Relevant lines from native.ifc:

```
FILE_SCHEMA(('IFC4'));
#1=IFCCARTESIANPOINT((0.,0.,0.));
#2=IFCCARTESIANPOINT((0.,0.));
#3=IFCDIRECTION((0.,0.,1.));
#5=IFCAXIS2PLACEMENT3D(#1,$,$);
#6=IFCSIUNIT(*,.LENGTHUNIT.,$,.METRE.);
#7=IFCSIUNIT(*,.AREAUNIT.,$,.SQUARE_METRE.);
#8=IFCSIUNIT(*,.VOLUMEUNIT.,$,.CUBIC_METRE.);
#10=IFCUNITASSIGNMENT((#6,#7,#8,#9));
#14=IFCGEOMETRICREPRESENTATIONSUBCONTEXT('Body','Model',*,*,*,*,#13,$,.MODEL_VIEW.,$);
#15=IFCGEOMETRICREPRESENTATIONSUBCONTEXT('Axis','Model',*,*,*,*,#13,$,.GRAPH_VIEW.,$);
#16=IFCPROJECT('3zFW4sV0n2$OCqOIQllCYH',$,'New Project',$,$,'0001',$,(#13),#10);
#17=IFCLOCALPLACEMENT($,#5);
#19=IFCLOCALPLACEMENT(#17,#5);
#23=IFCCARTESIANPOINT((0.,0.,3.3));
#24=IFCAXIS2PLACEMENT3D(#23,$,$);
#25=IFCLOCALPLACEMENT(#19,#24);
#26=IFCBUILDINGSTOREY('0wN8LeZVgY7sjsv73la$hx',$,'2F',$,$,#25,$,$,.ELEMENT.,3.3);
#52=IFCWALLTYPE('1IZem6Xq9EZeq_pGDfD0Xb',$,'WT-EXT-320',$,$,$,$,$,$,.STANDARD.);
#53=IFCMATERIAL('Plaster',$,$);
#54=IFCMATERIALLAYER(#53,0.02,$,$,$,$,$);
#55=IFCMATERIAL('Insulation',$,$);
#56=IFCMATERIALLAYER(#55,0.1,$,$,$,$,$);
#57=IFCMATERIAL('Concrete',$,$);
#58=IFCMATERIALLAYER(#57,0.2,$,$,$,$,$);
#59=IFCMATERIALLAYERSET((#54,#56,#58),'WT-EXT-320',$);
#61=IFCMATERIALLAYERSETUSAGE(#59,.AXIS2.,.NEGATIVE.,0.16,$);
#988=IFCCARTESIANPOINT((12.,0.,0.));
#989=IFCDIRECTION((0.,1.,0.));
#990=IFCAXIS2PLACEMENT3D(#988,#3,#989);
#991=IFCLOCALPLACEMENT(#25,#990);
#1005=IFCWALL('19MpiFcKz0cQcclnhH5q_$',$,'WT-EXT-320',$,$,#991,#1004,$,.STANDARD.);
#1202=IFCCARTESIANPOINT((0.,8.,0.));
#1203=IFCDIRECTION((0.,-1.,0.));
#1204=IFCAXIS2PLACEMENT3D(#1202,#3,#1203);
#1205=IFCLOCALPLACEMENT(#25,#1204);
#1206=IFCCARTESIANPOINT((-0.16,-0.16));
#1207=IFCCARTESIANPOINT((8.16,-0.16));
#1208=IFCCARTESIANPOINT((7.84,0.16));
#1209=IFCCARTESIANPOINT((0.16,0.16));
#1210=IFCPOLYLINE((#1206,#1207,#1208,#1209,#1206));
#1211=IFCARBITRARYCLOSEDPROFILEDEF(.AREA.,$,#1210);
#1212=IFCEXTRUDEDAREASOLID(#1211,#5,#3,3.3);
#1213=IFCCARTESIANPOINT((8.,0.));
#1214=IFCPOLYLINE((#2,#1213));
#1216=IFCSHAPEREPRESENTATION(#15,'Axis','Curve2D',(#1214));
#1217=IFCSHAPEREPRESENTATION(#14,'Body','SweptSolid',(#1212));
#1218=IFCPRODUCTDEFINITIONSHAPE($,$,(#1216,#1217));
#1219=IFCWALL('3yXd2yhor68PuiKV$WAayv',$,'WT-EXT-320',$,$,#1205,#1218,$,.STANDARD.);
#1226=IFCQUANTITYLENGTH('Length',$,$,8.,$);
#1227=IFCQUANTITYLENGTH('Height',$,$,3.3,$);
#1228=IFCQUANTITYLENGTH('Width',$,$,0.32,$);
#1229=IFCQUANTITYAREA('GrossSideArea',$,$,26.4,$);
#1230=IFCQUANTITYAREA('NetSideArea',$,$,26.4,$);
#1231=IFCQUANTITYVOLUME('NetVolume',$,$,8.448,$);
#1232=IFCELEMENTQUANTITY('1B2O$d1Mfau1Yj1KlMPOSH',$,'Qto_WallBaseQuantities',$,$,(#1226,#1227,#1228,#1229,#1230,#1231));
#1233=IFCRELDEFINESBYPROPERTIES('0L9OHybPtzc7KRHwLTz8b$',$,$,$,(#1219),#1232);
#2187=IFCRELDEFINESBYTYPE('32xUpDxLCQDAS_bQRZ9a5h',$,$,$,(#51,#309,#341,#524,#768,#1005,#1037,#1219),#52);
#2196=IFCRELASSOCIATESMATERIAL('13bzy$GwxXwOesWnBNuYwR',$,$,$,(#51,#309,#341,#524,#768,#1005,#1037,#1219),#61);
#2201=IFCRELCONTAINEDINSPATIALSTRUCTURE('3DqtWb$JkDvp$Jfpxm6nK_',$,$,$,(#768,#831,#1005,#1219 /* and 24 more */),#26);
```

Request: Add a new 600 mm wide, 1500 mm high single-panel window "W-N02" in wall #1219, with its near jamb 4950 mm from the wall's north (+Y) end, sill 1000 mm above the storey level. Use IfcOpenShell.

```python
import numpy as np
import ifcopenshell
import ifcopenshell.api.feature
import ifcopenshell.api.geometry
import ifcopenshell.api.pset
import ifcopenshell.api.root
import ifcopenshell.api.spatial
import ifcopenshell.geom
import ifcopenshell.util.element
import ifcopenshell.util.placement
import ifcopenshell.util.representation
import ifcopenshell.util.shape
import ifcopenshell.util.unit

model = ifcopenshell.open("native.ifc")
unit_scale = ifcopenshell.util.unit.calculate_unit_scale(model)
area_scale = ifcopenshell.util.unit.calculate_unit_scale(model, "AREAUNIT")
volume_scale = ifcopenshell.util.unit.calculate_unit_scale(model, "VOLUMEUNIT")
settings = ifcopenshell.geom.settings()


def volume(element):
    """Net volume in cubic metres, openings subtracted."""
    shape = ifcopenshell.geom.create_shape(settings, element)
    return ifcopenshell.util.shape.get_volume(shape.geometry)


wall = model.by_id(1219)
storey = ifcopenshell.util.element.get_container(wall, ifc_class="IfcBuildingStorey")
context = ifcopenshell.util.representation.get_context(model, "Model", "Body", "MODEL_VIEW")
before = volume(wall)

width, height, from_end, sill = 0.6, 1.5, 4.95, 1  # metres

# The wall runs along its own X axis, and the end named is its -X end.
wall_shape = ifcopenshell.geom.create_shape(settings, wall)
x, y, z = ifcopenshell.util.shape.get_vertices(wall_shape.geometry).T
start = x.min() + from_end
face, thickness = float(y.min()), float(y.max() - y.min())
wall_matrix = ifcopenshell.util.placement.get_local_placement(wall.ObjectPlacement)
level = ifcopenshell.util.placement.get_local_placement(storey.ObjectPlacement)[2, 3]


def in_wall(x, y):
    """Placement at x, y metres in the wall's axes, at sill height."""
    matrix = wall_matrix.copy()
    matrix[:, 3] = wall_matrix @ np.array([x / unit_scale, y / unit_scale, 0.0, 1.0])
    matrix[2, 3] = level + sill / unit_scale
    return matrix


# Opening: a box that overshoots both wall faces by 50 mm.
opening = ifcopenshell.api.root.create_entity(model, ifc_class="IfcOpeningElement", predefined_type="OPENING")
box = ifcopenshell.api.geometry.add_wall_representation(
    model, context=context, length=width, height=height, thickness=thickness + 0.1
)
ifcopenshell.api.geometry.assign_representation(model, product=opening, representation=box)
ifcopenshell.api.geometry.edit_object_placement(model, product=opening, matrix=in_wall(start, face - 0.05), is_si=False)
ifcopenshell.api.feature.add_feature(model, feature=opening, element=wall)

window = ifcopenshell.api.root.create_entity(model, ifc_class="IfcWindow", name="W-N02", predefined_type="WINDOW")
window.OverallWidth, window.OverallHeight = width / unit_scale, height / unit_scale
window.PartitioningType = "SINGLE_PANEL"
body = ifcopenshell.api.geometry.add_window_representation(
    model,
    context=context,
    overall_width=window.OverallWidth,
    overall_height=window.OverallHeight,
    partition_type="SINGLE_PANEL",
)
ifcopenshell.api.geometry.assign_representation(model, product=window, representation=body)
ifcopenshell.api.spatial.assign_container(model, products=[window], relating_structure=storey)
ifcopenshell.api.feature.add_filling(model, opening=opening, element=window)

# Centre the window in the wall's thickness.
ifcopenshell.api.geometry.edit_object_placement(model, product=window, matrix=in_wall(start, face), is_si=False)
window_shape = ifcopenshell.geom.create_shape(settings, window)
depth = ifcopenshell.util.shape.get_vertices(window_shape.geometry)[:, 1]
offset = face + thickness / 2 - (depth.min() + depth.max()) / 2
ifcopenshell.api.geometry.edit_object_placement(model, product=window, matrix=in_wall(start, offset), is_si=False)

after = volume(wall)

# Update the wall's stored quantities.
qto = model.by_id(ifcopenshell.util.element.get_pset(wall, "Qto_WallBaseQuantities", should_inherit=False)["id"])
ifcopenshell.api.pset.edit_qto(model, qto=qto, properties={
    "NetSideArea": after / thickness / area_scale,
    "NetVolume": after / volume_scale,
})

print(f"wall volume {before:.3f} -> {after:.3f} m3")

model.write("native_updated.ifc")
```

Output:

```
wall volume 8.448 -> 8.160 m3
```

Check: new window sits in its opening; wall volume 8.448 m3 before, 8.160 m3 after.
